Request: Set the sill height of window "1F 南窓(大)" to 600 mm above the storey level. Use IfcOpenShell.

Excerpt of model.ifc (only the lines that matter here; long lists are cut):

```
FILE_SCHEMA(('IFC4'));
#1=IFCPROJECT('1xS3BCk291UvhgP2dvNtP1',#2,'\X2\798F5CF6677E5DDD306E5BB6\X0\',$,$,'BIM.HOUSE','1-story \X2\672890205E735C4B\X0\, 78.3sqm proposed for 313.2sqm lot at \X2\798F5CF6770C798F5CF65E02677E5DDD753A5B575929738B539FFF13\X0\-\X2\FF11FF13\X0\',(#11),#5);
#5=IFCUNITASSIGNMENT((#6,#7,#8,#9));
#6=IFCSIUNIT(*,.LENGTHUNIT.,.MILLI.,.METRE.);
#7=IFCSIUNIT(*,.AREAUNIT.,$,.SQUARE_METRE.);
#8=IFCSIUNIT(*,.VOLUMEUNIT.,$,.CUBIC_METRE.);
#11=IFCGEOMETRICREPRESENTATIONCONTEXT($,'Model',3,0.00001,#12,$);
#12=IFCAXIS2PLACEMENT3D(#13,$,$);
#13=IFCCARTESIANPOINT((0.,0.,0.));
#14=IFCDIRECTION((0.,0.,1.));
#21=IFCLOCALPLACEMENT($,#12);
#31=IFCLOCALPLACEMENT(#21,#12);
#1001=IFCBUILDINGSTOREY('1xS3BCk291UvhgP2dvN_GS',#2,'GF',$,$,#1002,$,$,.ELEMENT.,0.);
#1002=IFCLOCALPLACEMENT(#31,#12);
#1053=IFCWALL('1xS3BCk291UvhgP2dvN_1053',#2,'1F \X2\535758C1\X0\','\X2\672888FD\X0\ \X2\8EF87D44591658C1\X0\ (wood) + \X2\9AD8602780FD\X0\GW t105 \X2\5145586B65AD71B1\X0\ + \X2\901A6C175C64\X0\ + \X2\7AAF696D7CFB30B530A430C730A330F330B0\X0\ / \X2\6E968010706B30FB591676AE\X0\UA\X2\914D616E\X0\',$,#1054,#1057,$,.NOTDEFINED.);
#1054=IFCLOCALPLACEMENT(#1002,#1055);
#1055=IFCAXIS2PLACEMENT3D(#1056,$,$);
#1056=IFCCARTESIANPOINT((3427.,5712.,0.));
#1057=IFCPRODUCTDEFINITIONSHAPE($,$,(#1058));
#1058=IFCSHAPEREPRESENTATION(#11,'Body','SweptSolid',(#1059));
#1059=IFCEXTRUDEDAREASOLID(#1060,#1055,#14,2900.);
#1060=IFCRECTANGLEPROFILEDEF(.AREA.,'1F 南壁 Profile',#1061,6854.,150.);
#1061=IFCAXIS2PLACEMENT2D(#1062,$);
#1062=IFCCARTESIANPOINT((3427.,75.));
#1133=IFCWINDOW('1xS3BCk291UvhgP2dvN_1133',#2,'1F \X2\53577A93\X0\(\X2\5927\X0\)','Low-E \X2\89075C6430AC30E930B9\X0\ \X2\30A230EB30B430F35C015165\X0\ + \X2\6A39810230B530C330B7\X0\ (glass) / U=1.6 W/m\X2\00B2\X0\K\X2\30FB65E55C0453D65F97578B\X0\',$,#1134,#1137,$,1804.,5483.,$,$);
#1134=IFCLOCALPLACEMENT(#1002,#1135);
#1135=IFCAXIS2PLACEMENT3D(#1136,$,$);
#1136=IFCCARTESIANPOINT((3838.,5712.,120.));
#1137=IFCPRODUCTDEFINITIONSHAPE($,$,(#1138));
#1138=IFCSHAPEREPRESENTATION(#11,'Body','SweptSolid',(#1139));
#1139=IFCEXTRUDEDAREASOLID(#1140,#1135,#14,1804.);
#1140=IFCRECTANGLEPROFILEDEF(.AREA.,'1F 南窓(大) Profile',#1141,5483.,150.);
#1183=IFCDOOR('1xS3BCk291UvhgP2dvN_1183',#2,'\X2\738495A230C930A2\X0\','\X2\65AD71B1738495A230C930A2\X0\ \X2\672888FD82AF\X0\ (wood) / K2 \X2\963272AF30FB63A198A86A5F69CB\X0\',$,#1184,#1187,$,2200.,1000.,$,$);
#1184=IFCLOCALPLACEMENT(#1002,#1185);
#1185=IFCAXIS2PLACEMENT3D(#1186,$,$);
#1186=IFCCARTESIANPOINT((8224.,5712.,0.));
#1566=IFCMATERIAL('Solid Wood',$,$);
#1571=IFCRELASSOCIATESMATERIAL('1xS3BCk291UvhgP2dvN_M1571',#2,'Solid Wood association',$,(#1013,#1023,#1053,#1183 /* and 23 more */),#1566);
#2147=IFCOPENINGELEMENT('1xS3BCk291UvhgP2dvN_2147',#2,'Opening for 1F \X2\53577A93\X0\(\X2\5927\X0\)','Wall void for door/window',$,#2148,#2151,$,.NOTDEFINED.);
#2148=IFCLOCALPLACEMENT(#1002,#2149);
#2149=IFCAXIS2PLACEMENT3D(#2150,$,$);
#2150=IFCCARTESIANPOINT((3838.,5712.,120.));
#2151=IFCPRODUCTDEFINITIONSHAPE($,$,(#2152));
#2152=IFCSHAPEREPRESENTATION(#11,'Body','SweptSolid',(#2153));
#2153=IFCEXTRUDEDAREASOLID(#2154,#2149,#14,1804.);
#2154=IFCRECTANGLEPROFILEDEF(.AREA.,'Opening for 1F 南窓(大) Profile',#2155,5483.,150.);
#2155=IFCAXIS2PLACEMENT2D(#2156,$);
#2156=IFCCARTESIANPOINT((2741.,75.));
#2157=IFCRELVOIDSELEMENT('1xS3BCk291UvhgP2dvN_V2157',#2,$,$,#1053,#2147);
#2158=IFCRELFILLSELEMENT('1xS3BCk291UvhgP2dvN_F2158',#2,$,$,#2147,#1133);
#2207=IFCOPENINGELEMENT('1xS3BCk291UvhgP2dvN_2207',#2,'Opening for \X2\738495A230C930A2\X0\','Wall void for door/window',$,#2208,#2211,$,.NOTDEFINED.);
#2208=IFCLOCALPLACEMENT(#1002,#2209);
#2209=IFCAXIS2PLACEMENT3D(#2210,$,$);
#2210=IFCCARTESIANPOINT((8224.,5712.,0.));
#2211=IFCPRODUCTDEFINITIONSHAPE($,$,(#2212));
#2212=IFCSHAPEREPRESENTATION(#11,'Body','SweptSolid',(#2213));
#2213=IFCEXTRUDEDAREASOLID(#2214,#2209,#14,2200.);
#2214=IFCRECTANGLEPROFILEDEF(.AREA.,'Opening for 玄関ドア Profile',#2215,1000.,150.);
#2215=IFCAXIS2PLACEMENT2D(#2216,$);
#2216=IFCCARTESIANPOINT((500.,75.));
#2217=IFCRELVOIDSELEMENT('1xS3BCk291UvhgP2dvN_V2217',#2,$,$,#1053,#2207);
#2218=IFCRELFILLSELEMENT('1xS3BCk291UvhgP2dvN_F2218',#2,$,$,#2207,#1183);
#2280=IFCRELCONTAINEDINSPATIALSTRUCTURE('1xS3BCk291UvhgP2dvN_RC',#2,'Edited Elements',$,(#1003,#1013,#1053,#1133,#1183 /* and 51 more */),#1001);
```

```python
import numpy as np
import ifcopenshell
import ifcopenshell.api.geometry
import ifcopenshell.geom
import ifcopenshell.util.element
import ifcopenshell.util.placement
import ifcopenshell.util.shape
import ifcopenshell.util.unit

model = ifcopenshell.open("model.ifc")
unit_scale = ifcopenshell.util.unit.calculate_unit_scale(model)

window = model.by_id(1133)
opening = window.FillsVoids[0].RelatingOpeningElement
storey = ifcopenshell.util.element.get_container(window, ifc_class="IfcBuildingStorey")
level = ifcopenshell.util.placement.get_local_placement(storey.ObjectPlacement)[2, 3]

# The opening's origin need not be at the sill, so measure its lowest point.
shape = ifcopenshell.geom.create_shape(ifcopenshell.geom.settings(), opening)
bottom = ifcopenshell.util.shape.get_shape_bottom_elevation(shape, shape.geometry) / unit_scale
dz = level + 0.6 / unit_scale - bottom

shift = np.array([0.0, 0.0, dz])
# The window is not placed relative to its opening, so move both.
for product in (opening, window):
    matrix = ifcopenshell.util.placement.get_local_placement(product.ObjectPlacement)
    matrix[:3, 3] += shift
    ifcopenshell.api.geometry.edit_object_placement(model, product=product, matrix=matrix, is_si=False)

print(f"moved by {dz * unit_scale:+.3f} m")

model.write("model_v2.ifc")
```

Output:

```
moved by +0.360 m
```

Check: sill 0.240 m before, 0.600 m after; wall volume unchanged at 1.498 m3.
